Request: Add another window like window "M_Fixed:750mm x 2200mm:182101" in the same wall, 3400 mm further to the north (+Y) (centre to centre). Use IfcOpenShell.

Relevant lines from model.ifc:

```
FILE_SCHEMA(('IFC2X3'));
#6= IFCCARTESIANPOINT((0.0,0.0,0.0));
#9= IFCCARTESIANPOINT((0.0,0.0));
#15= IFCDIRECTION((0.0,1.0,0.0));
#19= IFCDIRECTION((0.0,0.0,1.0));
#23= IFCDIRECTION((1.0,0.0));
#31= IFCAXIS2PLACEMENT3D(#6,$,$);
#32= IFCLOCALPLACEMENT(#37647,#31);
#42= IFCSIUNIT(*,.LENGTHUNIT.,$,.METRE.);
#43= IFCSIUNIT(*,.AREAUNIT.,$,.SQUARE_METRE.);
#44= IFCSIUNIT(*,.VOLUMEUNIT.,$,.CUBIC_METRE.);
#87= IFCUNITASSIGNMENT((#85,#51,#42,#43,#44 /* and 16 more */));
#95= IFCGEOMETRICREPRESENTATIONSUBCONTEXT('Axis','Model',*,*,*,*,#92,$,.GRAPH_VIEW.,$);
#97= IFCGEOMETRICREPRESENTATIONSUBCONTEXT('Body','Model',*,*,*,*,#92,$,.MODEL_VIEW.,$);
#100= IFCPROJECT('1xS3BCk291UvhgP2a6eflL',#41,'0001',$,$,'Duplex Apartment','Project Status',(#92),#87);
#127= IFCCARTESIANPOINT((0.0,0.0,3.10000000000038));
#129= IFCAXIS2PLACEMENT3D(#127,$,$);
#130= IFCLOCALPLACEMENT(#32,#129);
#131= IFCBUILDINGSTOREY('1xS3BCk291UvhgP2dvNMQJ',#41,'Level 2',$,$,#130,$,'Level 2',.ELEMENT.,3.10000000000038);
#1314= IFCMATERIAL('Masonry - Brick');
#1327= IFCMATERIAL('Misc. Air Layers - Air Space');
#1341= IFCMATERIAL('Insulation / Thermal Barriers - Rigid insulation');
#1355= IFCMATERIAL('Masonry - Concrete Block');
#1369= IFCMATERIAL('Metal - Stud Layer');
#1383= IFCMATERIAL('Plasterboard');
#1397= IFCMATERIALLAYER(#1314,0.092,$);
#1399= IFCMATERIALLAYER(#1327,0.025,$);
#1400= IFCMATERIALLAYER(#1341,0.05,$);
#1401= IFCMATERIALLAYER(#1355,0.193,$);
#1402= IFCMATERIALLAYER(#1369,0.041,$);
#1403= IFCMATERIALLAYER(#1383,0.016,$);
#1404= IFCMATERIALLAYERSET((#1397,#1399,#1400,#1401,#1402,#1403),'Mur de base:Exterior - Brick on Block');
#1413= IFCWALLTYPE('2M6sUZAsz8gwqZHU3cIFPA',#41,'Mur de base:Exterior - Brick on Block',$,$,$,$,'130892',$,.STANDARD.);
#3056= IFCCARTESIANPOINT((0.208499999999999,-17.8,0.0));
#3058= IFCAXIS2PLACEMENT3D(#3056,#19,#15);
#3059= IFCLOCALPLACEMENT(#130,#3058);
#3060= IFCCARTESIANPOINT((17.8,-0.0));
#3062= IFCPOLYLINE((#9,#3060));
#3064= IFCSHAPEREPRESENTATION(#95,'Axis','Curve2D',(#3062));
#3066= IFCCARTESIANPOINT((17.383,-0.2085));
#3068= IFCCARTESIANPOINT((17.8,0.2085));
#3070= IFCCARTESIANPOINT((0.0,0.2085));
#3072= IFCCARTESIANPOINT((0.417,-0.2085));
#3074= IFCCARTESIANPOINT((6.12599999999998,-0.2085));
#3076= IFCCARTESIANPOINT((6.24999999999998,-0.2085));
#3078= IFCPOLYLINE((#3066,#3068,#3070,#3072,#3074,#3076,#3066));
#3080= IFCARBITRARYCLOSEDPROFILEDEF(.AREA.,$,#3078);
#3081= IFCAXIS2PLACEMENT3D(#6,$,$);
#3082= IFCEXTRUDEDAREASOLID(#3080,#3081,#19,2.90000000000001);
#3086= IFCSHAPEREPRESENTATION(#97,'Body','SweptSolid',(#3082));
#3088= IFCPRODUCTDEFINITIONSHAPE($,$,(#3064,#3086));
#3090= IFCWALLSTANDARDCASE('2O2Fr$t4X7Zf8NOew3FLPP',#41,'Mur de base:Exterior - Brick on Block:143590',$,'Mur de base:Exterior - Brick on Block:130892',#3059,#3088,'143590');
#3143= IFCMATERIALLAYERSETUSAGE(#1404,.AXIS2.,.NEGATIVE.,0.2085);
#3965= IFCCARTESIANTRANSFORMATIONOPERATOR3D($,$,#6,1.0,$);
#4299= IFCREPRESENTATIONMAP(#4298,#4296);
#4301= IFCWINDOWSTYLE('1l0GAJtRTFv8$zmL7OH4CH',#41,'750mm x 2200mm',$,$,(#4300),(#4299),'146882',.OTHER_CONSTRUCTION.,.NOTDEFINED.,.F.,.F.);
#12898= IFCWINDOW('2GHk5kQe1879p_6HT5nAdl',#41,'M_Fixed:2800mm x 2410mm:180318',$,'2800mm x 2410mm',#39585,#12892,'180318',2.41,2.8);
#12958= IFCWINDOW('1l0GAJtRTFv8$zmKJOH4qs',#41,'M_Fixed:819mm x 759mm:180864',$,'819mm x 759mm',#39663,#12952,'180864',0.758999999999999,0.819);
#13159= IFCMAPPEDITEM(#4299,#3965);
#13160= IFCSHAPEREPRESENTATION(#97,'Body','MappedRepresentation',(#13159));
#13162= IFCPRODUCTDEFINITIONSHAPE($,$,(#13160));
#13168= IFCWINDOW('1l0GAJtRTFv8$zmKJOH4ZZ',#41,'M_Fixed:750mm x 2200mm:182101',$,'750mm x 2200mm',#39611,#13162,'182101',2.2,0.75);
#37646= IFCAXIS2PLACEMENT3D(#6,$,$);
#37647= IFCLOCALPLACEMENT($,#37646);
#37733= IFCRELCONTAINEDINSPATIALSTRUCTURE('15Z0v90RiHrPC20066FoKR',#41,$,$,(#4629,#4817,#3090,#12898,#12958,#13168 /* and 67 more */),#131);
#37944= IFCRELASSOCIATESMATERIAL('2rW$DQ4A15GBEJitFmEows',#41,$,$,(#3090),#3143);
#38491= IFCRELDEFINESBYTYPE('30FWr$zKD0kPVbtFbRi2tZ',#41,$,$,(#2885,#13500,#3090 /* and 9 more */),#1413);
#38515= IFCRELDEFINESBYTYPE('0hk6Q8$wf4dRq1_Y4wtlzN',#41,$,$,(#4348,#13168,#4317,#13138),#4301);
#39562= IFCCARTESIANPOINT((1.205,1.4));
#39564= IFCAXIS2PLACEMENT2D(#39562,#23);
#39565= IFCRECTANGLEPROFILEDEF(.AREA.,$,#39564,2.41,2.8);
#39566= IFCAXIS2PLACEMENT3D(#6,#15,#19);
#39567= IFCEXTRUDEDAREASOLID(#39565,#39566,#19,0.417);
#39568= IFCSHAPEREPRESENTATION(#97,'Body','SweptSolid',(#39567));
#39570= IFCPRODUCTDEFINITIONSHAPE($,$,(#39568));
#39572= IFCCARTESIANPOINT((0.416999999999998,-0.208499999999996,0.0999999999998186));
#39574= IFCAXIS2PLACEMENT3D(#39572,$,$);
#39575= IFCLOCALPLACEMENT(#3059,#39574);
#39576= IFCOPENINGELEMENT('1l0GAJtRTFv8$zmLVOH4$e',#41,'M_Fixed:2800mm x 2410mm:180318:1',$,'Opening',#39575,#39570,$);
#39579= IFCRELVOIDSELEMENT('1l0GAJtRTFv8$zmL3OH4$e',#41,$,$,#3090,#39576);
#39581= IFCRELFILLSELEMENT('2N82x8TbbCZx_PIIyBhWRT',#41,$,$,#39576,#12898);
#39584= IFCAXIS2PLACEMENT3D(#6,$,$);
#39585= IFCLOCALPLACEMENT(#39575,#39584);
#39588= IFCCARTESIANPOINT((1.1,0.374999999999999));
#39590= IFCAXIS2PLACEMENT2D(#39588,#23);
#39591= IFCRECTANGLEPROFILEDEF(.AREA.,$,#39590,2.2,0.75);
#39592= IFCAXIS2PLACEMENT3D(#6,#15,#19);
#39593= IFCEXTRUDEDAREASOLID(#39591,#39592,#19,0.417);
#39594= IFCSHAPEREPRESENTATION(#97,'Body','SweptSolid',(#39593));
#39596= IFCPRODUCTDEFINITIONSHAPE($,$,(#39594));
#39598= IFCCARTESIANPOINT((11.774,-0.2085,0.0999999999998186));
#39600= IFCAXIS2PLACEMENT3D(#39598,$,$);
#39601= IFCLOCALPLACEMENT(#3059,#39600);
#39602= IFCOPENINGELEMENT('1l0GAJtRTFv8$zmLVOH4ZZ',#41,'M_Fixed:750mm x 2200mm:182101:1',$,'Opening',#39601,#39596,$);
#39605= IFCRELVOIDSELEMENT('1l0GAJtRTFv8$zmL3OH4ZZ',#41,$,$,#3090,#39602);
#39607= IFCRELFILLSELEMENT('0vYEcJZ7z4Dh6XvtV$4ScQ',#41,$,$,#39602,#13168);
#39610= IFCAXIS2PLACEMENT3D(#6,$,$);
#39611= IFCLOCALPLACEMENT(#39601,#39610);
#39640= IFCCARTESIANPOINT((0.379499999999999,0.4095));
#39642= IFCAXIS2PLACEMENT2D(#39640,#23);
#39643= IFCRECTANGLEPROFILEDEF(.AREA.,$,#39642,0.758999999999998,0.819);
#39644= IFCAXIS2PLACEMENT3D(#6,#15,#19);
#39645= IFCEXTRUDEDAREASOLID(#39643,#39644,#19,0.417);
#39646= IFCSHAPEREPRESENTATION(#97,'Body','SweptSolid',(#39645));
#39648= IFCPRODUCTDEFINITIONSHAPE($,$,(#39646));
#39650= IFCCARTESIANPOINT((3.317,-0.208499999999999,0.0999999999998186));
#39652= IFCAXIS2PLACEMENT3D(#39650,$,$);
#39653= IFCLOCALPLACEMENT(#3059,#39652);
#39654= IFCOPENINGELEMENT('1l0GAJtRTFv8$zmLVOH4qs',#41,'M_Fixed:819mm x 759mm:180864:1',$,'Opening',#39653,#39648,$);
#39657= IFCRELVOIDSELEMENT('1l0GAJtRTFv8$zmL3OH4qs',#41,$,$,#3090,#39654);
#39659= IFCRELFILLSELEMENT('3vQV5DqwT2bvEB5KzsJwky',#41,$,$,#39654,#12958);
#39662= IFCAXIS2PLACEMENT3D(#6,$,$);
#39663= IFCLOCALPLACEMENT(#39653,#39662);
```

```python
import ifcopenshell
import ifcopenshell.api.feature
import ifcopenshell.api.geometry
import ifcopenshell.api.root
import ifcopenshell.geom
import ifcopenshell.util.element
import ifcopenshell.util.placement
import ifcopenshell.util.shape
import ifcopenshell.util.unit

model = ifcopenshell.open("model.ifc")
unit_scale = ifcopenshell.util.unit.calculate_unit_scale(model)
settings = ifcopenshell.geom.settings()


def volume(element):
    """Net volume in cubic metres, openings subtracted."""
    shape = ifcopenshell.geom.create_shape(settings, element)
    return ifcopenshell.util.shape.get_volume(shape.geometry)


def reuse_history(source, copy):
    """copy_class also copies each property set's owner history, people and application; keep the originals."""
    for rel in copy.IsDefinedBy:
        if rel.is_a("IfcRelDefinesByProperties") and (history := rel.RelatingPropertyDefinition.OwnerHistory):
            rel.RelatingPropertyDefinition.OwnerHistory = source.OwnerHistory
            ifcopenshell.util.element.remove_deep2(model, history)


window = model.by_guid("1l0GAJtRTFv8$zmKJOH4ZZ")
opening = window.FillsVoids[0].RelatingOpeningElement
wall = opening.VoidsElements[0].RelatingBuildingElement
before = volume(wall)
shift = ifcopenshell.util.placement.get_local_placement(wall.ObjectPlacement)[:3, 0] * 3.4 / unit_scale

# copy_class copies the void relationship, type, container and properties, but no geometry.
new_opening = ifcopenshell.api.root.copy_class(model, product=opening)
new_opening.Representation = ifcopenshell.util.element.copy_deep(
    model, opening.Representation, exclude=["IfcGeometricRepresentationContext", "IfcRepresentationMap"]
)
new_opening.Name = "M_Fixed:750mm x 2200mm"
new_window = ifcopenshell.api.root.copy_class(model, product=window)
new_window.Representation = ifcopenshell.util.element.copy_deep(
    model, window.Representation, exclude=["IfcGeometricRepresentationContext", "IfcRepresentationMap"]
)
new_window.Name = "M_Fixed:750mm x 2200mm"
new_window.Tag = None
reuse_history(window, new_window)
fills = ifcopenshell.api.feature.add_filling(model, opening=new_opening, element=new_window)
fills.OwnerHistory = new_window.OwnerHistory  # required in IFC2X3

for old, new in ((opening, new_opening), (window, new_window)):
    matrix = ifcopenshell.util.placement.get_local_placement(old.ObjectPlacement)
    matrix[:3, 3] += shift
    ifcopenshell.api.geometry.edit_object_placement(model, product=new, matrix=matrix, is_si=False)

after = volume(wall)

print(f"wall volume {before:.3f} -> {after:.3f} m3")

model.write("model_rev.ifc")
```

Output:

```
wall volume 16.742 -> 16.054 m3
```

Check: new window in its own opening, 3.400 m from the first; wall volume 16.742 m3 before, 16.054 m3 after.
